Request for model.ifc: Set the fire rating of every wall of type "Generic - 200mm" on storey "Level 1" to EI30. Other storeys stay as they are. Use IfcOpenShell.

First a look at what the model holds.

```python
import ifcopenshell
import ifcopenshell.util.element

model = ifcopenshell.open("model.ifc")
print(model.schema)
storey = next(s for s in model.by_type("IfcBuildingStorey") if s.Name == "Level 1")
walls = [e for e in ifcopenshell.util.element.get_decomposition(storey) if e.is_a("IfcWall")]
seen = {}
for e in walls:
    element_type = ifcopenshell.util.element.get_type(e)
    key = (element_type.Name if element_type != e and element_type else None, ifcopenshell.util.element.get_pset(e, "Pset_WallCommon", "FireRating"))
    seen[key] = seen.get(key, 0) + 1
for (name, value), count in sorted(seen.items(), key=str):
    print(count, "x", name, "|", value)
```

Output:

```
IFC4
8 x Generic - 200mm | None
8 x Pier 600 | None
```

```python
import ifcopenshell
import ifcopenshell.api.pset
import ifcopenshell.util.element

model = ifcopenshell.open("model.ifc")

storey = next(s for s in model.by_type("IfcBuildingStorey") if s.Name == "Level 1")
walls = [e for e in ifcopenshell.util.element.get_decomposition(storey) if e.is_a("IfcWall")]

count = 0
for e in walls:
    element_type = ifcopenshell.util.element.get_type(e)
    if element_type in (None, e) or element_type.Name != "Generic - 200mm":
        continue
    # add_pset returns the element's existing set when there is one.
    pset = ifcopenshell.api.pset.add_pset(model, product=e, name="Pset_WallCommon")
    ifcopenshell.api.pset.edit_pset(model, pset=pset, properties={"FireRating": "EI30"})
    count += 1

print(count, "walls updated")

model.write("model_rev.ifc")
```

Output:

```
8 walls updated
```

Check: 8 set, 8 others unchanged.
